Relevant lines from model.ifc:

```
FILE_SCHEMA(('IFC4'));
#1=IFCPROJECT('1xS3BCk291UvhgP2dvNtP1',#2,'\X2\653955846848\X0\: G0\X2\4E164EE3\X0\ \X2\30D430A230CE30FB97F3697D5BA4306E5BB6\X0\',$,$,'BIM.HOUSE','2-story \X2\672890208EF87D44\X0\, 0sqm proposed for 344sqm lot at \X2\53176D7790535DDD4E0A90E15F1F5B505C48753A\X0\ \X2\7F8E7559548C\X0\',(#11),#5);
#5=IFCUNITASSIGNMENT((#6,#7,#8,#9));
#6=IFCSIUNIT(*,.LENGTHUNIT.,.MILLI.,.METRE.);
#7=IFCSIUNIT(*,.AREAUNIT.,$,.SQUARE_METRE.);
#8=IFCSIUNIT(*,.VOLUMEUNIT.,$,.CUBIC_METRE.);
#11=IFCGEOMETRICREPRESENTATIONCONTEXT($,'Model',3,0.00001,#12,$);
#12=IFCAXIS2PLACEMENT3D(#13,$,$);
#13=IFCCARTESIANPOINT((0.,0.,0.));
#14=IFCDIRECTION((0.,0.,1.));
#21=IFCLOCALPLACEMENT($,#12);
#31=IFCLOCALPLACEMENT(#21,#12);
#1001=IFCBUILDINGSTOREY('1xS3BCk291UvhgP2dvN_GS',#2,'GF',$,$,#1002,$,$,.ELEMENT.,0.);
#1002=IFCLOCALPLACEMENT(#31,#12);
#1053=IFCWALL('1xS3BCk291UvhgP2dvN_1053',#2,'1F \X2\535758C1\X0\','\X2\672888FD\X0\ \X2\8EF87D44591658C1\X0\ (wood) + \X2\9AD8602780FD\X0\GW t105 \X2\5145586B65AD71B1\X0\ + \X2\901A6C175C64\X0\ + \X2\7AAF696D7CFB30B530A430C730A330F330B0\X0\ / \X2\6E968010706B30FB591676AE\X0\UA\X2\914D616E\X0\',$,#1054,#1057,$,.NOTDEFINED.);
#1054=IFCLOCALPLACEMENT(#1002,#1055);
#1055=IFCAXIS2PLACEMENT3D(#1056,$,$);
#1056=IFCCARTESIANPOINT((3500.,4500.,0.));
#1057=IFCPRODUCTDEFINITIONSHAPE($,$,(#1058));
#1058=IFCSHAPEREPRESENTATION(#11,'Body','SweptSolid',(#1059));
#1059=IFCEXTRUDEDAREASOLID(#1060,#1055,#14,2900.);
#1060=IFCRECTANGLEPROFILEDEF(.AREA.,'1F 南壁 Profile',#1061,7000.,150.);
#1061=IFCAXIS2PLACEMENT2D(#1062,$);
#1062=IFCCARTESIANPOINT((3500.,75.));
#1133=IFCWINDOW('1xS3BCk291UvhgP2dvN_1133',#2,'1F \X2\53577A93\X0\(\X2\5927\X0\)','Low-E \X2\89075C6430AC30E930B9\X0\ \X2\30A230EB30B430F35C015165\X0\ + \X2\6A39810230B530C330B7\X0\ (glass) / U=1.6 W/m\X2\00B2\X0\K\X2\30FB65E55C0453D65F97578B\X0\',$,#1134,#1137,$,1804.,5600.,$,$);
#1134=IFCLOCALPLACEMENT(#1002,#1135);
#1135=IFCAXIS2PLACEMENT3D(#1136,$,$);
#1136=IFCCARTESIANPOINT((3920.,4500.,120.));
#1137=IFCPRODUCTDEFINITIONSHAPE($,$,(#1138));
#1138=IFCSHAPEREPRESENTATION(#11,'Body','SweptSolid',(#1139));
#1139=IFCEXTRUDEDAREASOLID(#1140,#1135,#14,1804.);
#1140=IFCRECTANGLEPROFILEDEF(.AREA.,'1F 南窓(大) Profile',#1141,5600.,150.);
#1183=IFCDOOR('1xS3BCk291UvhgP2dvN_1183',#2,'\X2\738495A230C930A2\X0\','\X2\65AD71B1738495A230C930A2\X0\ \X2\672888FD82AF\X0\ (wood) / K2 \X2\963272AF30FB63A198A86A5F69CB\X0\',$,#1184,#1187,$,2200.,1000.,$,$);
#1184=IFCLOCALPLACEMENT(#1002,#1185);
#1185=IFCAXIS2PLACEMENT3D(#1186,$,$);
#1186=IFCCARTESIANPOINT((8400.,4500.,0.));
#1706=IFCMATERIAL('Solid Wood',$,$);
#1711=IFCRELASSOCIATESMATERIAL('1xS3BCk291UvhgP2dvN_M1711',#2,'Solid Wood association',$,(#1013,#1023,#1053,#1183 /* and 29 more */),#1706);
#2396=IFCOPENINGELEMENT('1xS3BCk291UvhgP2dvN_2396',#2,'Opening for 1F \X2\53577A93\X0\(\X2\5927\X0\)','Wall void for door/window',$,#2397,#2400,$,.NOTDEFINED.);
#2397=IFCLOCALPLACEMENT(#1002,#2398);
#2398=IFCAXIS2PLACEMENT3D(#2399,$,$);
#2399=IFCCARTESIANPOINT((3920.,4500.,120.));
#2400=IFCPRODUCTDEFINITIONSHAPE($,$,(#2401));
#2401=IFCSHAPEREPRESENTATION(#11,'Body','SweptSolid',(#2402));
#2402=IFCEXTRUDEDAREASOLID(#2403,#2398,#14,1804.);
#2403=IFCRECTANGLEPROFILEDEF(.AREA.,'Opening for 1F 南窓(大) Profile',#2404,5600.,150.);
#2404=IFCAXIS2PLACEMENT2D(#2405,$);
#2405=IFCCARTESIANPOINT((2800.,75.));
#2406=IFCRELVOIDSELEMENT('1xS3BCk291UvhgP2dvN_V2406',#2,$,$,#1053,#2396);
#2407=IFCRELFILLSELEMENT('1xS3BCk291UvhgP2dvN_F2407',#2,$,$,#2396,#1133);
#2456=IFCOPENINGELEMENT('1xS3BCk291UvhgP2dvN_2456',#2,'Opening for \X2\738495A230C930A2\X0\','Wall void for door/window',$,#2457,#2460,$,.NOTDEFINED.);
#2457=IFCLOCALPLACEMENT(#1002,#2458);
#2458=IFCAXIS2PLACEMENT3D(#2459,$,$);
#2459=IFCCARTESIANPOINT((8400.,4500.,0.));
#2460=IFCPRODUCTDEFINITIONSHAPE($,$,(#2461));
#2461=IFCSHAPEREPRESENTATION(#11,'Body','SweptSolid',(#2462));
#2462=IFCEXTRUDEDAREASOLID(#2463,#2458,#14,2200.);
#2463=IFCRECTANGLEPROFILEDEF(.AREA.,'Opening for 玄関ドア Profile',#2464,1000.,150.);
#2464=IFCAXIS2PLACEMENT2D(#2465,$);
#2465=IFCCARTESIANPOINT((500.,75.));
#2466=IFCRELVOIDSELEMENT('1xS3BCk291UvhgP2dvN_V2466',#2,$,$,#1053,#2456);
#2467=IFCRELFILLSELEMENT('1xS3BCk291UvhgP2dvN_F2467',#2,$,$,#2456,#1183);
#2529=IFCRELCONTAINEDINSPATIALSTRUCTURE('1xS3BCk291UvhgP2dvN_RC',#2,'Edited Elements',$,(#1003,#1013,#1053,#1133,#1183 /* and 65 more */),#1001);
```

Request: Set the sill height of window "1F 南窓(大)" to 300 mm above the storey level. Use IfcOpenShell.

```python
import numpy as np
import ifcopenshell
import ifcopenshell.api.geometry
import ifcopenshell.geom
import ifcopenshell.util.element
import ifcopenshell.util.placement
import ifcopenshell.util.shape
import ifcopenshell.util.unit

model = ifcopenshell.open("model.ifc")
unit_scale = ifcopenshell.util.unit.calculate_unit_scale(model)

window = model.by_guid("1xS3BCk291UvhgP2dvN_1133")
opening = window.FillsVoids[0].RelatingOpeningElement
storey = ifcopenshell.util.element.get_container(window, ifc_class="IfcBuildingStorey")
level = ifcopenshell.util.placement.get_local_placement(storey.ObjectPlacement)[2, 3]

# The opening's origin need not be at the sill, so measure its lowest point.
shape = ifcopenshell.geom.create_shape(ifcopenshell.geom.settings(), opening)
bottom = ifcopenshell.util.shape.get_shape_bottom_elevation(shape, shape.geometry) / unit_scale
dz = level + 300.0 - bottom

shift = np.array([0.0, 0.0, dz])
# The window is not placed relative to its opening, so move both.
for product in (opening, window):
    matrix = ifcopenshell.util.placement.get_local_placement(product.ObjectPlacement)
    matrix[:3, 3] += shift
    ifcopenshell.api.geometry.edit_object_placement(model, product=product, matrix=matrix, is_si=False)

print(f"moved by {dz * unit_scale:+.3f} m")

model.write("model_v2.ifc")
```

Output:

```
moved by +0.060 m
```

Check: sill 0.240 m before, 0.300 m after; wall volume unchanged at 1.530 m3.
